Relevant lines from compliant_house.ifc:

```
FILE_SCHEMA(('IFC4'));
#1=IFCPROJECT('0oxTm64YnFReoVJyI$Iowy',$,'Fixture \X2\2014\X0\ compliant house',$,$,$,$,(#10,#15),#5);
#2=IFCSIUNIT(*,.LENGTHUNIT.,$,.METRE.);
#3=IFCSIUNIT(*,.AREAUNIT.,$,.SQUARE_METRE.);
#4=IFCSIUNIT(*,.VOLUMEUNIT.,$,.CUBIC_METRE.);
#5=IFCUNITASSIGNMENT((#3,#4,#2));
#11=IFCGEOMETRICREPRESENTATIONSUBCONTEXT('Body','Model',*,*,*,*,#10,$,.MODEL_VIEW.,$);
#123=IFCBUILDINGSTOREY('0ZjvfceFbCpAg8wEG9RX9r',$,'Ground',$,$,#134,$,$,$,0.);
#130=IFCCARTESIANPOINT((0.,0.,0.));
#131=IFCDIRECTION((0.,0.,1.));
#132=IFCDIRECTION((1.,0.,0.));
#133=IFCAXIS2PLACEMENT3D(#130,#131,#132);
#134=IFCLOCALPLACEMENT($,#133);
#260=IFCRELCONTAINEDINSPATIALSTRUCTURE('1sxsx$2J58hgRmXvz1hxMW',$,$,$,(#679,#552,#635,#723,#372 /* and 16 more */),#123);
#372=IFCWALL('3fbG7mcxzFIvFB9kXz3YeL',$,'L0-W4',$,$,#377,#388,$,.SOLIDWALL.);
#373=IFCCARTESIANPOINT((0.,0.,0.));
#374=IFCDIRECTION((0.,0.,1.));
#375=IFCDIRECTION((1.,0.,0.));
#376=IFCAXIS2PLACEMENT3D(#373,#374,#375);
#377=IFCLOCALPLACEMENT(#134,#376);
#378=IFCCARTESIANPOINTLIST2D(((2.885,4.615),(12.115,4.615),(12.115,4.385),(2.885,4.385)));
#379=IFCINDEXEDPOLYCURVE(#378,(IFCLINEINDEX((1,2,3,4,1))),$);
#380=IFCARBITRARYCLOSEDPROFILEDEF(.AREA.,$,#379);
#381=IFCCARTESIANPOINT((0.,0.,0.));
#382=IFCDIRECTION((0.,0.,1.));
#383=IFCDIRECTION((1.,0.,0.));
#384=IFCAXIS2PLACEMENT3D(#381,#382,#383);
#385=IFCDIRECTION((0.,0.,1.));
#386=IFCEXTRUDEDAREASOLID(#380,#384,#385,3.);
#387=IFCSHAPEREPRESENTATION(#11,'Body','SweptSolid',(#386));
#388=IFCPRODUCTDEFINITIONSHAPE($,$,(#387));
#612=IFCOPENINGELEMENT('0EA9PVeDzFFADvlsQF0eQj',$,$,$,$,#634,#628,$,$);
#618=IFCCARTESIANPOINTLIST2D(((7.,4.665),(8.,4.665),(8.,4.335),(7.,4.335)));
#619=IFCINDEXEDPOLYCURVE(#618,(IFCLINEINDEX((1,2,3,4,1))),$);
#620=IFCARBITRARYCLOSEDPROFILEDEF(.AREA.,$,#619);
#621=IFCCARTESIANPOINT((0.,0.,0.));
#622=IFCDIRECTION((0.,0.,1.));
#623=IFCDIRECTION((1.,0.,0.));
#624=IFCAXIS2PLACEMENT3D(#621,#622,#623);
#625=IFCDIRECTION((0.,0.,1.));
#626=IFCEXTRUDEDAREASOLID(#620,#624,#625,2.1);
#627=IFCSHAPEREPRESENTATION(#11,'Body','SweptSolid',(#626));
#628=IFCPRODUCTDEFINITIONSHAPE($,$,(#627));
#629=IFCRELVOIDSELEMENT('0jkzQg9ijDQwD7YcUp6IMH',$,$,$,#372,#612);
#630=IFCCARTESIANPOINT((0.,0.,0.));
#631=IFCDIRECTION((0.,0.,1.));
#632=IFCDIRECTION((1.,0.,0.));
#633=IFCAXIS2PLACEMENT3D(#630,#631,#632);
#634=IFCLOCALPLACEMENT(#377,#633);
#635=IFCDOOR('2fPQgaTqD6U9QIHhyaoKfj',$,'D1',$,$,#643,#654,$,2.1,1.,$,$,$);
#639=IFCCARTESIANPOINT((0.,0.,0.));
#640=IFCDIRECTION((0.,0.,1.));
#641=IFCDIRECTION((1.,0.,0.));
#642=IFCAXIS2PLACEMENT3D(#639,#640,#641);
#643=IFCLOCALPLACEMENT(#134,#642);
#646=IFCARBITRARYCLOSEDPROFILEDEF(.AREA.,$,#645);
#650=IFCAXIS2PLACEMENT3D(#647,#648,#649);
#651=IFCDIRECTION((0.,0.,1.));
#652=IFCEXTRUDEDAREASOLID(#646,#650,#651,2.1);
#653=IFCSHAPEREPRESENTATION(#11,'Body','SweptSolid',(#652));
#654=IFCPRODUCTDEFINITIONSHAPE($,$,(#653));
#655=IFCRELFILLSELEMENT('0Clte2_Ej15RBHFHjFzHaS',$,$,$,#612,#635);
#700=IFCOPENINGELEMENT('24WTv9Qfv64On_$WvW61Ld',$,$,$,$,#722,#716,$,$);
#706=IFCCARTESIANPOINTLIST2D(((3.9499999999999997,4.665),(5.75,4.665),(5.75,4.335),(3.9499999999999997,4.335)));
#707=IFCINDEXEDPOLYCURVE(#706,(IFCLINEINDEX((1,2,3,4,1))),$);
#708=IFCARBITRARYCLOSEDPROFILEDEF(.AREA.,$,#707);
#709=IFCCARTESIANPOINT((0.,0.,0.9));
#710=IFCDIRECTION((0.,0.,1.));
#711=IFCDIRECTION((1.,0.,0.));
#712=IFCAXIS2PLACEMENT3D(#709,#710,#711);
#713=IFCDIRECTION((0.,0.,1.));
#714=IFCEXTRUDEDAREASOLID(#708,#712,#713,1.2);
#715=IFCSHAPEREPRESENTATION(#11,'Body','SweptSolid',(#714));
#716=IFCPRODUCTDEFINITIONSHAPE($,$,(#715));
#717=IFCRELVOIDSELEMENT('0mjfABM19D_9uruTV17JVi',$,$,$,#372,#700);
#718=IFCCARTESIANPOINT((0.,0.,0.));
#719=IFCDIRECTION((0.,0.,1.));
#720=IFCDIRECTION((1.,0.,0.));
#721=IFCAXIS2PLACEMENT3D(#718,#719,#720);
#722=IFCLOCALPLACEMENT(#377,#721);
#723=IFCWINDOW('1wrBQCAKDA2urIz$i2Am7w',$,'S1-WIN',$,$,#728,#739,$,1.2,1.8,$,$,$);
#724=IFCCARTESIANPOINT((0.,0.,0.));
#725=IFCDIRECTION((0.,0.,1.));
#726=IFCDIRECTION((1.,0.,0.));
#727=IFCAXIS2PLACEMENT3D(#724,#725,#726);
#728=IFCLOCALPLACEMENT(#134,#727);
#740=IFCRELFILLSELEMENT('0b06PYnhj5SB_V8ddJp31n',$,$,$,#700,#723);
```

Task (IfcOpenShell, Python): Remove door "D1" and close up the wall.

```python
import ifcopenshell
import ifcopenshell.api.feature
import ifcopenshell.api.root
import ifcopenshell.geom
import ifcopenshell.util.shape

model = ifcopenshell.open("compliant_house.ifc")
settings = ifcopenshell.geom.settings()


def volume(element):
    """Net volume in cubic metres, openings subtracted."""
    shape = ifcopenshell.geom.create_shape(settings, element)
    return ifcopenshell.util.shape.get_volume(shape.geometry)


door = model.by_guid("2fPQgaTqD6U9QIHhyaoKfj")
opening = door.FillsVoids[0].RelatingOpeningElement
wall = opening.VoidsElements[0].RelatingBuildingElement
before = volume(wall)

ifcopenshell.api.root.remove_product(model, product=door)
ifcopenshell.api.feature.remove_feature(model, feature=opening)

after = volume(wall)

print(f"wall volume {before:.3f} -> {after:.3f} m3")

model.write("compliant_house-out.ifc")
```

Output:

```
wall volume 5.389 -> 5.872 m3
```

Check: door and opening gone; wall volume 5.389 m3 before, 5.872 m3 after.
